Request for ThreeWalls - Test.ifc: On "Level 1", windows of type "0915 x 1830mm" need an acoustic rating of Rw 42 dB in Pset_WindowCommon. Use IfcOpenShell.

First a look at what the model holds.

```python
import ifcopenshell
import ifcopenshell.util.element

model = ifcopenshell.open("ThreeWalls - Test.ifc")
print(model.schema)
storey = next(s for s in model.by_type("IfcBuildingStorey") if s.Name == "Level 1")
windows = [e for e in ifcopenshell.util.element.get_decomposition(storey) if e.is_a("IfcWindow")]
seen = {}
for e in windows:
    element_type = ifcopenshell.util.element.get_type(e)
    key = (element_type.Name if element_type != e and element_type else None, ifcopenshell.util.element.get_pset(e, "Pset_WindowCommon", "AcousticRating"))
    seen[key] = seen.get(key, 0) + 1
for (name, value), count in sorted(seen.items(), key=str):
    print(count, "x", name, "|", value)
```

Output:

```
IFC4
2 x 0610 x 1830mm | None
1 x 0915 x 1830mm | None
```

```python
import ifcopenshell
import ifcopenshell.api.pset
import ifcopenshell.util.element

model = ifcopenshell.open("ThreeWalls - Test.ifc")

storey = next(s for s in model.by_type("IfcBuildingStorey") if s.Name == "Level 1")
windows = [e for e in ifcopenshell.util.element.get_decomposition(storey) if e.is_a("IfcWindow")]

count = 0
for e in windows:
    element_type = ifcopenshell.util.element.get_type(e)
    if element_type in (None, e) or element_type.Name != "0915 x 1830mm":
        continue
    # add_pset returns the element's existing set when there is one.
    pset = ifcopenshell.api.pset.add_pset(model, product=e, name="Pset_WindowCommon")
    ifcopenshell.api.pset.edit_pset(model, pset=pset, properties={"AcousticRating": "Rw 42 dB"})
    count += 1

print(count, "windows updated")

model.write("ThreeWalls - Test_updated.ifc")
```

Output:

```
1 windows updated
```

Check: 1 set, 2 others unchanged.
